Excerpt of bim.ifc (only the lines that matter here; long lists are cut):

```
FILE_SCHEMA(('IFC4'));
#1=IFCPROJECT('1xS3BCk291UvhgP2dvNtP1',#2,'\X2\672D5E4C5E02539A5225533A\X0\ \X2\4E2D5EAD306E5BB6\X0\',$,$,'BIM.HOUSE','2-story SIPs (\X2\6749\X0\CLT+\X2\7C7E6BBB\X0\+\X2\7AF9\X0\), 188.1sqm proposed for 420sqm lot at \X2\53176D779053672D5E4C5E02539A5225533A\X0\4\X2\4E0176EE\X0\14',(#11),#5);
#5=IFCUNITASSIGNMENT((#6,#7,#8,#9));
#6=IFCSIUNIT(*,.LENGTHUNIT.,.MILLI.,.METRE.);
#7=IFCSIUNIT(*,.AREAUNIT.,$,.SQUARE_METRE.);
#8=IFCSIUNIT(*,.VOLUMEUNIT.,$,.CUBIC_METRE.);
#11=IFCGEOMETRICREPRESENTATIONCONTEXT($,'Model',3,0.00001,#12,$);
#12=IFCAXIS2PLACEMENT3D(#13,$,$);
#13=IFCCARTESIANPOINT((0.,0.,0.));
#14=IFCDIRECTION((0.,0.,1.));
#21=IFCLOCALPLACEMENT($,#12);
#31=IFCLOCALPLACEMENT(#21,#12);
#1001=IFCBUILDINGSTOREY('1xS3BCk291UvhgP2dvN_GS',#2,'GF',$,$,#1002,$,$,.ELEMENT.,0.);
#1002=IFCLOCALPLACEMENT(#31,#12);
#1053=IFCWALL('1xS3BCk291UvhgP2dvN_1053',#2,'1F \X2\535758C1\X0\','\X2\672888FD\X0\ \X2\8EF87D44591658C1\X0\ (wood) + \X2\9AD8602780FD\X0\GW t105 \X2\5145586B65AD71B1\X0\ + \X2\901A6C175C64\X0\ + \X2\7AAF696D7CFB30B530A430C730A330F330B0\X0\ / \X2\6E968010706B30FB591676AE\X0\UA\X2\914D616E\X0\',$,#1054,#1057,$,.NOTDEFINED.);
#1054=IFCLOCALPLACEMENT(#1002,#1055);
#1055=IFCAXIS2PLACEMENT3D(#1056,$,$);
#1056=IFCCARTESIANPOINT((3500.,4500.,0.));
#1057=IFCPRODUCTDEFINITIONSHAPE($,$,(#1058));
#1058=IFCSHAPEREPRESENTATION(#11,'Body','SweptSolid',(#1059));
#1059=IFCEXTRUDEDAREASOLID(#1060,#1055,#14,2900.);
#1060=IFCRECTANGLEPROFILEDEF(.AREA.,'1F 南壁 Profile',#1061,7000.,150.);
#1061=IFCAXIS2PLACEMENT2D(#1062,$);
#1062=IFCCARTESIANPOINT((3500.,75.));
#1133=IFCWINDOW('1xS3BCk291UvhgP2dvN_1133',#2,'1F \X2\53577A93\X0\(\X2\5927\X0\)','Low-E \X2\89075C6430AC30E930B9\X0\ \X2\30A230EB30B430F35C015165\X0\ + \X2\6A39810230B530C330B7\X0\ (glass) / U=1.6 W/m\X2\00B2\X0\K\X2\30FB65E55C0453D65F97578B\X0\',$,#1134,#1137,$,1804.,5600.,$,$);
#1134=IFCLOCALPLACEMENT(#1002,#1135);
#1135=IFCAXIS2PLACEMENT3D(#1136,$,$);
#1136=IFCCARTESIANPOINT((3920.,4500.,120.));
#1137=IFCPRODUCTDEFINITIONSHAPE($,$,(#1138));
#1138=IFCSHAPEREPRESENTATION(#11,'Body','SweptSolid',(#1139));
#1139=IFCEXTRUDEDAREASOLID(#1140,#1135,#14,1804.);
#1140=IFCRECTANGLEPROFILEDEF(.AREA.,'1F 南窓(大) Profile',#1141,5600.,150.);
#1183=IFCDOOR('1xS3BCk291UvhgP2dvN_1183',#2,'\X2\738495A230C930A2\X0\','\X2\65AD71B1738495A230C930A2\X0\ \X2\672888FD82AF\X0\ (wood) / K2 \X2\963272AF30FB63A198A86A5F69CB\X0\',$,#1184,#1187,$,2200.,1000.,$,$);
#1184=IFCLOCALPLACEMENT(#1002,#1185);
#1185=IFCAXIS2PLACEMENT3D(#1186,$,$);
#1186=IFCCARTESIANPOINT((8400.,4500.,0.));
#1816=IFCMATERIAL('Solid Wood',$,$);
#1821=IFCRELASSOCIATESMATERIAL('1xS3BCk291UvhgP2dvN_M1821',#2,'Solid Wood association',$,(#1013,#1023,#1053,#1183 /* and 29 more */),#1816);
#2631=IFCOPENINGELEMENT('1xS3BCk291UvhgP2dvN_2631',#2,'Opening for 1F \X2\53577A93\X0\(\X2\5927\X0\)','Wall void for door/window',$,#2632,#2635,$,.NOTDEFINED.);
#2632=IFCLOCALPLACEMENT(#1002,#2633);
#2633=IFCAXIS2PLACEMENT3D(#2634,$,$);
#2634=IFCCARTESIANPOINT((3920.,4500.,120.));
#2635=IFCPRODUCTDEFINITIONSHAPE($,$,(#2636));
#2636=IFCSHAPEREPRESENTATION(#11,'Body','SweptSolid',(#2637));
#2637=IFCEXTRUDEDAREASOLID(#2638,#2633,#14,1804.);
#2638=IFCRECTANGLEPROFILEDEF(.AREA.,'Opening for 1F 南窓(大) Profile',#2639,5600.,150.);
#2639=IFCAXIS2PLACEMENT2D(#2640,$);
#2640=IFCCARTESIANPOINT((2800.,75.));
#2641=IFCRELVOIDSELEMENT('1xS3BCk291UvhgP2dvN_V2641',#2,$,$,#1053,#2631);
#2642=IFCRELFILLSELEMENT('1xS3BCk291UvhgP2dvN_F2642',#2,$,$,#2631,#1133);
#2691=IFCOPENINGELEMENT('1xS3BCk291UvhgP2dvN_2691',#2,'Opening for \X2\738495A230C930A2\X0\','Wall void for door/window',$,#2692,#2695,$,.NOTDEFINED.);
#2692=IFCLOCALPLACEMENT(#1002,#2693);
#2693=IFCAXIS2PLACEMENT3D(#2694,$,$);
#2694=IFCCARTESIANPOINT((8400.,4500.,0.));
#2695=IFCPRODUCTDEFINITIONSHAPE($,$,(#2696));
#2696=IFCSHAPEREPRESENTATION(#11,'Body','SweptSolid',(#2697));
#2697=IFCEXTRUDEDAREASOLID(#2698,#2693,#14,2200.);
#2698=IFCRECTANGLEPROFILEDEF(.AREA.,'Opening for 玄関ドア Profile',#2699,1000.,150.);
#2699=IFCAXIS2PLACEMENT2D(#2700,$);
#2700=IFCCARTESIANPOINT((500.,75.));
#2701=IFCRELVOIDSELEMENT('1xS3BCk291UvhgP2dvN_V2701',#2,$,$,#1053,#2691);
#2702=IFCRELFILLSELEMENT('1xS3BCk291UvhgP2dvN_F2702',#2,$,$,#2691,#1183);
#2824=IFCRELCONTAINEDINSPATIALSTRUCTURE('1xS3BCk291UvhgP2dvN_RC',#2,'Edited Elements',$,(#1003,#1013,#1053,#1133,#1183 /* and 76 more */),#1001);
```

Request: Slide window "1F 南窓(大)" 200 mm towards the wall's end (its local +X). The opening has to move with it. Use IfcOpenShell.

```python
import ifcopenshell
import ifcopenshell.api.geometry
import ifcopenshell.util.placement

model = ifcopenshell.open("bim.ifc")

window = model.by_id(1133)
opening = window.FillsVoids[0].RelatingOpeningElement
wall = opening.VoidsElements[0].RelatingBuildingElement

wall_matrix = ifcopenshell.util.placement.get_local_placement(wall.ObjectPlacement)
shift = wall_matrix[:3, 0] * 200.0
before = ifcopenshell.util.placement.get_local_placement(window.ObjectPlacement)[:3, 3].copy()

# The window is not placed relative to its opening, so move both.
for product in (opening, window):
    matrix = ifcopenshell.util.placement.get_local_placement(product.ObjectPlacement)
    matrix[:3, 3] += shift
    ifcopenshell.api.geometry.edit_object_placement(model, product=product, matrix=matrix, is_si=False)

after = ifcopenshell.util.placement.get_local_placement(window.ObjectPlacement)[:3, 3]
print("window moved by", (after - before).round(3) + 0.0)

model.write("bim-out.ifc")
```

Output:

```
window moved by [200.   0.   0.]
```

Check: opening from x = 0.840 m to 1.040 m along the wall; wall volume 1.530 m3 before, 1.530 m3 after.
